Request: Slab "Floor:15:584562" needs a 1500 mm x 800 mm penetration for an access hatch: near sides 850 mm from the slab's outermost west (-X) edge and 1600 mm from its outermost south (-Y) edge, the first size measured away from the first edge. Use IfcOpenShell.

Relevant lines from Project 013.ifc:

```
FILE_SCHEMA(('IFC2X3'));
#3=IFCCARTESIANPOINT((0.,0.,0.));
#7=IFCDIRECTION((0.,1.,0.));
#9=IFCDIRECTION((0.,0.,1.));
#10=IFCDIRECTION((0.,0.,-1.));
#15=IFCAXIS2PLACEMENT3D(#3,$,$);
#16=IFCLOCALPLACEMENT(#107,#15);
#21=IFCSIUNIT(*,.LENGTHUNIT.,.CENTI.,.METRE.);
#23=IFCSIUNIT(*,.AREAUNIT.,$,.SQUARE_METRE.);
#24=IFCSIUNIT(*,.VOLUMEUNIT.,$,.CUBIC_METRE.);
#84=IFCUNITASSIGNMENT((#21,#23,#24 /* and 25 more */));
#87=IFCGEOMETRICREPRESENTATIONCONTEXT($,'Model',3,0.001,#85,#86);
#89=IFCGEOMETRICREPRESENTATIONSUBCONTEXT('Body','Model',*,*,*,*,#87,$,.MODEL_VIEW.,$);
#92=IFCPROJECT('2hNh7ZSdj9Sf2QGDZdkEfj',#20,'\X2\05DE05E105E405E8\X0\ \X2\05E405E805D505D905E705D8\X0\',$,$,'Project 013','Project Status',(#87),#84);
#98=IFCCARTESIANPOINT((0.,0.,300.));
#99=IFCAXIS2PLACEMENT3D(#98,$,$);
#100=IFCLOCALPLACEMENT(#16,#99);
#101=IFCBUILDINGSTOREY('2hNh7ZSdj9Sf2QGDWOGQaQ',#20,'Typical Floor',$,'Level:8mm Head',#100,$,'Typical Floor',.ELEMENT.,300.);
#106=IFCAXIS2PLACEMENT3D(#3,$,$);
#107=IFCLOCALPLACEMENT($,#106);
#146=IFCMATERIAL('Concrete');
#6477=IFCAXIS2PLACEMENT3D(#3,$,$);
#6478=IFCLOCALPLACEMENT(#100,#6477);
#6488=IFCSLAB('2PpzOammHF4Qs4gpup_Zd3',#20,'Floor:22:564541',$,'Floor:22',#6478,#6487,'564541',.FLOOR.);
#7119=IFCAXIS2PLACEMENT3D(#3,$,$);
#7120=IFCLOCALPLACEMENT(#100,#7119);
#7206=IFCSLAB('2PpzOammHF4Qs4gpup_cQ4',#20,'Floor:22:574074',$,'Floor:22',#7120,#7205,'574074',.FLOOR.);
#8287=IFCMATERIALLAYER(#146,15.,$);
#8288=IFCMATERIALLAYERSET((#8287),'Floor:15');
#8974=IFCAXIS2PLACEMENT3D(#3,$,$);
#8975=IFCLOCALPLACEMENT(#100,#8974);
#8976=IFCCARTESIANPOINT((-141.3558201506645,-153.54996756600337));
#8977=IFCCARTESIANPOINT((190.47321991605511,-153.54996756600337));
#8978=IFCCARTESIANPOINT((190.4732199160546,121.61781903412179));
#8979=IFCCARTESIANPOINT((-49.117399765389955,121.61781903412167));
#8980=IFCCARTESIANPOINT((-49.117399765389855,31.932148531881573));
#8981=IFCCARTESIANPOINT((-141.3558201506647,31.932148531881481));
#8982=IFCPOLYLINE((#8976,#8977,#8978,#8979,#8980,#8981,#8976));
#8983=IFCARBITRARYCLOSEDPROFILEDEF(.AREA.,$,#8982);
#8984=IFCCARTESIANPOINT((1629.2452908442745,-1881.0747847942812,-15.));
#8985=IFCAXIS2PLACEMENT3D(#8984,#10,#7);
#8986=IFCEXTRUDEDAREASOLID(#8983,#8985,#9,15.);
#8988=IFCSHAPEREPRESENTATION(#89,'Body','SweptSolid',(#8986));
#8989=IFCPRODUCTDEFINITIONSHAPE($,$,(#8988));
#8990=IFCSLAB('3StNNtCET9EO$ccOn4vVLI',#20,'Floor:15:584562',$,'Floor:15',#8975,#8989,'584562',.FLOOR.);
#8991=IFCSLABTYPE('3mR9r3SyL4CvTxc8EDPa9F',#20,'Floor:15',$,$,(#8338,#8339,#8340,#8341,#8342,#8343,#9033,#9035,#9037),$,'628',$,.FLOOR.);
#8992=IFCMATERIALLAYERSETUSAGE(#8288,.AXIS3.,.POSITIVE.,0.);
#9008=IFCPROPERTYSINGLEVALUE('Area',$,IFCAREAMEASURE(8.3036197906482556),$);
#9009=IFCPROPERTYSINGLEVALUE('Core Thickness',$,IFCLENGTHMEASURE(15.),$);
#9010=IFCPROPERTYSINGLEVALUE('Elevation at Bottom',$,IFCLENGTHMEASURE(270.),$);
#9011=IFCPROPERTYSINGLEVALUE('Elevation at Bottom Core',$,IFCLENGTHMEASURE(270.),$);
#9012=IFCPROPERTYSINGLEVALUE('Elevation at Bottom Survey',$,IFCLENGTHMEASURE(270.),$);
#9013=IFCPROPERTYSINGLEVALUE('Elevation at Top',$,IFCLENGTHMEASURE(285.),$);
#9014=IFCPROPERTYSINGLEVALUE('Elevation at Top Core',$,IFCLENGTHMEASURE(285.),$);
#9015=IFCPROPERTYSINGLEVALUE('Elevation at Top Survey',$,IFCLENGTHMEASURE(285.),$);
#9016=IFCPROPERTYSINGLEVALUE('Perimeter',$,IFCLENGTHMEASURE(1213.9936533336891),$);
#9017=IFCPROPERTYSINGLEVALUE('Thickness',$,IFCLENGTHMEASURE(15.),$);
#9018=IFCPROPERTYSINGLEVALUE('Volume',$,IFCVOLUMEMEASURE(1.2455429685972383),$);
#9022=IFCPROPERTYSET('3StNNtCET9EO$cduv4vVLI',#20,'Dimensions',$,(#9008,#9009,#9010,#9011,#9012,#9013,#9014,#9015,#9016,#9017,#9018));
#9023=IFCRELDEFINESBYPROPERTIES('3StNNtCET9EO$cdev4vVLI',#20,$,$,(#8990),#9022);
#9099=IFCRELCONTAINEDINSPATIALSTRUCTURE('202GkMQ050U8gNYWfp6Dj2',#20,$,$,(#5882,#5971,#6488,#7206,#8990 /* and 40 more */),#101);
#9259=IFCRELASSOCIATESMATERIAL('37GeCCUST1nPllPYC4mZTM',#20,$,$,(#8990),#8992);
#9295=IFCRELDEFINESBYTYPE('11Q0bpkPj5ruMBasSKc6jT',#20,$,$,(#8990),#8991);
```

```python
import numpy as np
import ifcopenshell
import ifcopenshell.api.feature
import ifcopenshell.api.geometry
import ifcopenshell.api.pset
import ifcopenshell.api.root
import ifcopenshell.geom
import ifcopenshell.util.element
import ifcopenshell.util.placement
import ifcopenshell.util.representation
import ifcopenshell.util.shape
import ifcopenshell.util.unit

model = ifcopenshell.open("Project 013.ifc")
unit_scale = ifcopenshell.util.unit.calculate_unit_scale(model)
area_scale = ifcopenshell.util.unit.calculate_unit_scale(model, "AREAUNIT")
volume_scale = ifcopenshell.util.unit.calculate_unit_scale(model, "VOLUMEUNIT")
settings = ifcopenshell.geom.settings()


def volume(element):
    """Net volume in cubic metres, openings subtracted."""
    shape = ifcopenshell.geom.create_shape(settings, element)
    return ifcopenshell.util.shape.get_volume(shape.geometry)


slab = model.by_id(8990)
before = volume(slab)

# Extent in the slab's own axes, in metres. The edges named are its -X and -Y sides.
slab_shape = ifcopenshell.geom.create_shape(settings, slab)
vertices = ifcopenshell.util.shape.get_vertices(slab_shape.geometry)
x_min, y_min, bottom = vertices.min(axis=0)
top = vertices[:, 2].max()

opening = ifcopenshell.api.root.create_entity(model, ifc_class="IfcOpeningElement", name="Access hatch opening")
context = ifcopenshell.util.representation.get_context(model, "Model", "Body", "MODEL_VIEW")
width, depth = 1.5, 0.8
outline = [(0.0, 0.0), (width, 0.0), (width, depth), (0.0, depth), (0.0, 0.0)]
# Overshoot both faces by 50 mm so the cut is clean.
shape = ifcopenshell.api.geometry.add_slab_representation(
    model, context=context, depth=top - bottom + 0.1, polyline=outline
)
ifcopenshell.api.geometry.assign_representation(model, product=opening, representation=shape)

matrix = ifcopenshell.util.placement.get_local_placement(slab.ObjectPlacement)
matrix[:, 3] = matrix @ np.append(np.array([x_min + 0.85, y_min + 1.6, bottom - 0.05]) / unit_scale, 1.0)
ifcopenshell.api.geometry.edit_object_placement(model, product=opening, matrix=matrix, is_si=False)
ifcopenshell.api.feature.add_feature(model, feature=opening, element=slab)

after = volume(slab)

# Update the slab's stored quantities.
pset = model.by_id(ifcopenshell.util.element.get_pset(slab, "Dimensions", should_inherit=False)["id"])
ifcopenshell.api.pset.edit_pset(model, pset=pset, properties={
    "Area": model.create_entity("IfcAreaMeasure", after / (top - bottom) / area_scale),
    "Volume": model.create_entity("IfcVolumeMeasure", after / volume_scale),
})

print(f"slab volume {before:.3f} -> {after:.3f} m3")

model.write("Project 013_rev.ifc")
```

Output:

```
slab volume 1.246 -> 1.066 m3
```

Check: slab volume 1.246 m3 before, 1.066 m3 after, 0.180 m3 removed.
